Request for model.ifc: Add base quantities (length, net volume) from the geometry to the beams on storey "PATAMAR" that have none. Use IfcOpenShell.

First a look at what the model holds.

```python
import ifcopenshell
import ifcopenshell.util.element
import ifcopenshell.util.unit

model = ifcopenshell.open("model.ifc")
print(model.schema)
for unit_type in ("LENGTHUNIT", "AREAUNIT", "VOLUMEUNIT"):
    print(unit_type, ifcopenshell.util.unit.calculate_unit_scale(model, unit_type))
storey = next(s for s in model.by_type("IfcBuildingStorey") if s.Name == "PATAMAR")
beams = [e for e in ifcopenshell.util.element.get_decomposition(storey) if e.is_a("IfcBeam")]
for e in sorted(beams, key=lambda e: e.id()):
    print(e.id(), e.is_a(), e.Name, list(ifcopenshell.util.element.get_psets(e, qtos_only=True)), sep=" | ")
```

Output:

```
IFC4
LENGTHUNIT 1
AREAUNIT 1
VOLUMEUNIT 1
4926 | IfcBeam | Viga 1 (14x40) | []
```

```python
import ifcopenshell
import ifcopenshell.api.pset
import ifcopenshell.geom
import ifcopenshell.util.element
import ifcopenshell.util.shape
import ifcopenshell.util.unit

model = ifcopenshell.open("model.ifc")
unit_scale = ifcopenshell.util.unit.calculate_unit_scale(model)
volume_scale = ifcopenshell.util.unit.calculate_unit_scale(model, "VOLUMEUNIT")
settings = ifcopenshell.geom.settings()

storey = next(s for s in model.by_type("IfcBuildingStorey") if s.Name == "PATAMAR")
beams = [e for e in ifcopenshell.util.element.get_decomposition(storey) if e.is_a("IfcBeam")]

for e in sorted(beams, key=lambda e: e.id()):
    if ifcopenshell.util.element.get_psets(e, qtos_only=True, should_inherit=False):
        continue
    # Geometry comes back in metres, in the element's own axes.
    shape = ifcopenshell.geom.create_shape(settings, e)
    values = {
        "Length": ifcopenshell.util.shape.get_max_xyz(shape.geometry) / unit_scale,
        "NetVolume": ifcopenshell.util.shape.get_volume(shape.geometry) / volume_scale,
    }
    qto = ifcopenshell.api.pset.add_qto(model, product=e, name="Qto_BeamBaseQuantities")
    ifcopenshell.api.pset.edit_qto(model, qto=qto, properties=values)
    print(e.id(), {k: round(v, 3) for k, v in values.items()})

model.write("model_edited.ifc")
```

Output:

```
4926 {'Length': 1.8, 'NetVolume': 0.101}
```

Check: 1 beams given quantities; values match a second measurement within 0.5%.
